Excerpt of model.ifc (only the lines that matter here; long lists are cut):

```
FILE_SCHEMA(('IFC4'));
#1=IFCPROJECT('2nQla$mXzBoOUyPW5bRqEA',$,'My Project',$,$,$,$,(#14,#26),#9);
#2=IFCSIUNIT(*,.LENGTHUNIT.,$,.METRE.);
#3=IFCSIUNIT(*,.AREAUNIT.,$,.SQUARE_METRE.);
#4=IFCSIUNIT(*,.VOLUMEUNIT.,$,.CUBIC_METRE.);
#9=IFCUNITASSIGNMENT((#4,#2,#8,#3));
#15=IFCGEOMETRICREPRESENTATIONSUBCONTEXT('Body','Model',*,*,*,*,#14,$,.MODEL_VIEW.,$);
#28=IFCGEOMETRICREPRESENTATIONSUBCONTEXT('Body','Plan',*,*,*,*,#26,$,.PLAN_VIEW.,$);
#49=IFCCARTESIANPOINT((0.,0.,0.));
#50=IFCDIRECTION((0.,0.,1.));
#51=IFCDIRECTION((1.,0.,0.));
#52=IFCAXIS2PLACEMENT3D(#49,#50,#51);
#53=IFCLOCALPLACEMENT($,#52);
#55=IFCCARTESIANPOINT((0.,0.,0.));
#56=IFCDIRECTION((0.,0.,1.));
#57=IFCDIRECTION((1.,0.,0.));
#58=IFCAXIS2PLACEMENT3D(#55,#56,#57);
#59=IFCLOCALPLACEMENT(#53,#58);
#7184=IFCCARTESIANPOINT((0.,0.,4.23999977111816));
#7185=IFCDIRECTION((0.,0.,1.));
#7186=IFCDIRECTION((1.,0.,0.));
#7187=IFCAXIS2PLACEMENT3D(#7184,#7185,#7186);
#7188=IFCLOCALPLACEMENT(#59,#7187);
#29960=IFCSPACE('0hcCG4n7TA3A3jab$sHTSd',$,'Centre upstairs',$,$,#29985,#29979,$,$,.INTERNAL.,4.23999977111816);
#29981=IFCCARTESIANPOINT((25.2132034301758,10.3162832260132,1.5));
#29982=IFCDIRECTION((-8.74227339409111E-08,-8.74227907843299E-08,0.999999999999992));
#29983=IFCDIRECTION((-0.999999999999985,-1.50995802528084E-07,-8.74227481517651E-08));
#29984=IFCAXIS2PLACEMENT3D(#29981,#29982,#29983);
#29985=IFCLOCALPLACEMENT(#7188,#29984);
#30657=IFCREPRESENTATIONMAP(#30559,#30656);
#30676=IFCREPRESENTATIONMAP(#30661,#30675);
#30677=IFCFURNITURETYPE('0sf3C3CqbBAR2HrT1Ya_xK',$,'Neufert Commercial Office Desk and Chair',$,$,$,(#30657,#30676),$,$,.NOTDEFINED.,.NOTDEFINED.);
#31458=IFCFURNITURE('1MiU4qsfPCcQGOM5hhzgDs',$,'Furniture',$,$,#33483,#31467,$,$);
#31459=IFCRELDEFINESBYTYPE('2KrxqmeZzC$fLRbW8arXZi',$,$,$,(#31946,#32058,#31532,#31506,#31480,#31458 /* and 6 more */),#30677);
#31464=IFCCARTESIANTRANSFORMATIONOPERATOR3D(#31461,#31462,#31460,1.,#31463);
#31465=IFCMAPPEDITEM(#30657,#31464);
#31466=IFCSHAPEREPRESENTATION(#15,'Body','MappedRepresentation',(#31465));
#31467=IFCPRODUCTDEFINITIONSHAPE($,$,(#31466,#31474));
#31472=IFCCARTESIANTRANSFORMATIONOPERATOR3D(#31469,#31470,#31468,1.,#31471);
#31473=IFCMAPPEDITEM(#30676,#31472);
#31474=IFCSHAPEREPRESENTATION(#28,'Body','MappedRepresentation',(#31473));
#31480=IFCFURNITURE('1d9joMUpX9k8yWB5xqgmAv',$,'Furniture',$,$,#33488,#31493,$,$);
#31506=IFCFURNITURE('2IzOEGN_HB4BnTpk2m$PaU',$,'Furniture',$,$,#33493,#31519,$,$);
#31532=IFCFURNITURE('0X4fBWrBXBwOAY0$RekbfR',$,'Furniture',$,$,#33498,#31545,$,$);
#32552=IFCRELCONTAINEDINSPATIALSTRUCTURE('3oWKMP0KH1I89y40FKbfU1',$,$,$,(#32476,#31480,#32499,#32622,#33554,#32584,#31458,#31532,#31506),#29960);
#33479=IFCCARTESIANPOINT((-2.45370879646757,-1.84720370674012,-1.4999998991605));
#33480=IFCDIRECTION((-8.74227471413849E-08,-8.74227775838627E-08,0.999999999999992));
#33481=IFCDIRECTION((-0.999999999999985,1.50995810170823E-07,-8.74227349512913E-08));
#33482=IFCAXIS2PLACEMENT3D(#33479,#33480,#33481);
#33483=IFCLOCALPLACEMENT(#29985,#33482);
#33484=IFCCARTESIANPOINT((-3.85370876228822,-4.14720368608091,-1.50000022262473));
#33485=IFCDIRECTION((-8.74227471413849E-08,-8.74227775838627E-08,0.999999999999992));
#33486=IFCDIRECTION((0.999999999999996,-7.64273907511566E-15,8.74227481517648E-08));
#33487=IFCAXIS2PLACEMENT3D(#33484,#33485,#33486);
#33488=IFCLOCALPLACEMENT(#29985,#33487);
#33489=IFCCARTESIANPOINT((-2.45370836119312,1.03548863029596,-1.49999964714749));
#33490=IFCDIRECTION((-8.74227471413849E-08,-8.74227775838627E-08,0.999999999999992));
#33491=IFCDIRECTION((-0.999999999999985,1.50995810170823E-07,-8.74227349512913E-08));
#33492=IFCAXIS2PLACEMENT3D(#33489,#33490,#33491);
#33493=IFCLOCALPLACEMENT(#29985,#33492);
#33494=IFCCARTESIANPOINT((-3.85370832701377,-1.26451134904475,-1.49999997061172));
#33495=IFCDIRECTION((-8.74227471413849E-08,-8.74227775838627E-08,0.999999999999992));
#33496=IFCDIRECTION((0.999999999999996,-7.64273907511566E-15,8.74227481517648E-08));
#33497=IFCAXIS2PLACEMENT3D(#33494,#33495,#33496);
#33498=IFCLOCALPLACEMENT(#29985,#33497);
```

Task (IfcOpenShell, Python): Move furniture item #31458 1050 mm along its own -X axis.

```python
import ifcopenshell
import ifcopenshell.api.geometry
import ifcopenshell.util.placement
import ifcopenshell.util.unit

model = ifcopenshell.open("model.ifc")
unit_scale = ifcopenshell.util.unit.calculate_unit_scale(model)

item = model.by_id(31458)
matrix = ifcopenshell.util.placement.get_local_placement(item.ObjectPlacement)
matrix[:3, 3] -= matrix[:3, 0] * 1.05 / unit_scale
ifcopenshell.api.geometry.edit_object_placement(model, product=item, matrix=matrix, is_si=False)

print(ifcopenshell.util.placement.get_local_placement(item.ObjectPlacement).round(3) + 0.0)

model.write("model-out.ifc")
```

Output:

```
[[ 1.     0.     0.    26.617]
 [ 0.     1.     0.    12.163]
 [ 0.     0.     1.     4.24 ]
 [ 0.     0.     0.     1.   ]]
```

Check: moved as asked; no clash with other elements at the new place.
